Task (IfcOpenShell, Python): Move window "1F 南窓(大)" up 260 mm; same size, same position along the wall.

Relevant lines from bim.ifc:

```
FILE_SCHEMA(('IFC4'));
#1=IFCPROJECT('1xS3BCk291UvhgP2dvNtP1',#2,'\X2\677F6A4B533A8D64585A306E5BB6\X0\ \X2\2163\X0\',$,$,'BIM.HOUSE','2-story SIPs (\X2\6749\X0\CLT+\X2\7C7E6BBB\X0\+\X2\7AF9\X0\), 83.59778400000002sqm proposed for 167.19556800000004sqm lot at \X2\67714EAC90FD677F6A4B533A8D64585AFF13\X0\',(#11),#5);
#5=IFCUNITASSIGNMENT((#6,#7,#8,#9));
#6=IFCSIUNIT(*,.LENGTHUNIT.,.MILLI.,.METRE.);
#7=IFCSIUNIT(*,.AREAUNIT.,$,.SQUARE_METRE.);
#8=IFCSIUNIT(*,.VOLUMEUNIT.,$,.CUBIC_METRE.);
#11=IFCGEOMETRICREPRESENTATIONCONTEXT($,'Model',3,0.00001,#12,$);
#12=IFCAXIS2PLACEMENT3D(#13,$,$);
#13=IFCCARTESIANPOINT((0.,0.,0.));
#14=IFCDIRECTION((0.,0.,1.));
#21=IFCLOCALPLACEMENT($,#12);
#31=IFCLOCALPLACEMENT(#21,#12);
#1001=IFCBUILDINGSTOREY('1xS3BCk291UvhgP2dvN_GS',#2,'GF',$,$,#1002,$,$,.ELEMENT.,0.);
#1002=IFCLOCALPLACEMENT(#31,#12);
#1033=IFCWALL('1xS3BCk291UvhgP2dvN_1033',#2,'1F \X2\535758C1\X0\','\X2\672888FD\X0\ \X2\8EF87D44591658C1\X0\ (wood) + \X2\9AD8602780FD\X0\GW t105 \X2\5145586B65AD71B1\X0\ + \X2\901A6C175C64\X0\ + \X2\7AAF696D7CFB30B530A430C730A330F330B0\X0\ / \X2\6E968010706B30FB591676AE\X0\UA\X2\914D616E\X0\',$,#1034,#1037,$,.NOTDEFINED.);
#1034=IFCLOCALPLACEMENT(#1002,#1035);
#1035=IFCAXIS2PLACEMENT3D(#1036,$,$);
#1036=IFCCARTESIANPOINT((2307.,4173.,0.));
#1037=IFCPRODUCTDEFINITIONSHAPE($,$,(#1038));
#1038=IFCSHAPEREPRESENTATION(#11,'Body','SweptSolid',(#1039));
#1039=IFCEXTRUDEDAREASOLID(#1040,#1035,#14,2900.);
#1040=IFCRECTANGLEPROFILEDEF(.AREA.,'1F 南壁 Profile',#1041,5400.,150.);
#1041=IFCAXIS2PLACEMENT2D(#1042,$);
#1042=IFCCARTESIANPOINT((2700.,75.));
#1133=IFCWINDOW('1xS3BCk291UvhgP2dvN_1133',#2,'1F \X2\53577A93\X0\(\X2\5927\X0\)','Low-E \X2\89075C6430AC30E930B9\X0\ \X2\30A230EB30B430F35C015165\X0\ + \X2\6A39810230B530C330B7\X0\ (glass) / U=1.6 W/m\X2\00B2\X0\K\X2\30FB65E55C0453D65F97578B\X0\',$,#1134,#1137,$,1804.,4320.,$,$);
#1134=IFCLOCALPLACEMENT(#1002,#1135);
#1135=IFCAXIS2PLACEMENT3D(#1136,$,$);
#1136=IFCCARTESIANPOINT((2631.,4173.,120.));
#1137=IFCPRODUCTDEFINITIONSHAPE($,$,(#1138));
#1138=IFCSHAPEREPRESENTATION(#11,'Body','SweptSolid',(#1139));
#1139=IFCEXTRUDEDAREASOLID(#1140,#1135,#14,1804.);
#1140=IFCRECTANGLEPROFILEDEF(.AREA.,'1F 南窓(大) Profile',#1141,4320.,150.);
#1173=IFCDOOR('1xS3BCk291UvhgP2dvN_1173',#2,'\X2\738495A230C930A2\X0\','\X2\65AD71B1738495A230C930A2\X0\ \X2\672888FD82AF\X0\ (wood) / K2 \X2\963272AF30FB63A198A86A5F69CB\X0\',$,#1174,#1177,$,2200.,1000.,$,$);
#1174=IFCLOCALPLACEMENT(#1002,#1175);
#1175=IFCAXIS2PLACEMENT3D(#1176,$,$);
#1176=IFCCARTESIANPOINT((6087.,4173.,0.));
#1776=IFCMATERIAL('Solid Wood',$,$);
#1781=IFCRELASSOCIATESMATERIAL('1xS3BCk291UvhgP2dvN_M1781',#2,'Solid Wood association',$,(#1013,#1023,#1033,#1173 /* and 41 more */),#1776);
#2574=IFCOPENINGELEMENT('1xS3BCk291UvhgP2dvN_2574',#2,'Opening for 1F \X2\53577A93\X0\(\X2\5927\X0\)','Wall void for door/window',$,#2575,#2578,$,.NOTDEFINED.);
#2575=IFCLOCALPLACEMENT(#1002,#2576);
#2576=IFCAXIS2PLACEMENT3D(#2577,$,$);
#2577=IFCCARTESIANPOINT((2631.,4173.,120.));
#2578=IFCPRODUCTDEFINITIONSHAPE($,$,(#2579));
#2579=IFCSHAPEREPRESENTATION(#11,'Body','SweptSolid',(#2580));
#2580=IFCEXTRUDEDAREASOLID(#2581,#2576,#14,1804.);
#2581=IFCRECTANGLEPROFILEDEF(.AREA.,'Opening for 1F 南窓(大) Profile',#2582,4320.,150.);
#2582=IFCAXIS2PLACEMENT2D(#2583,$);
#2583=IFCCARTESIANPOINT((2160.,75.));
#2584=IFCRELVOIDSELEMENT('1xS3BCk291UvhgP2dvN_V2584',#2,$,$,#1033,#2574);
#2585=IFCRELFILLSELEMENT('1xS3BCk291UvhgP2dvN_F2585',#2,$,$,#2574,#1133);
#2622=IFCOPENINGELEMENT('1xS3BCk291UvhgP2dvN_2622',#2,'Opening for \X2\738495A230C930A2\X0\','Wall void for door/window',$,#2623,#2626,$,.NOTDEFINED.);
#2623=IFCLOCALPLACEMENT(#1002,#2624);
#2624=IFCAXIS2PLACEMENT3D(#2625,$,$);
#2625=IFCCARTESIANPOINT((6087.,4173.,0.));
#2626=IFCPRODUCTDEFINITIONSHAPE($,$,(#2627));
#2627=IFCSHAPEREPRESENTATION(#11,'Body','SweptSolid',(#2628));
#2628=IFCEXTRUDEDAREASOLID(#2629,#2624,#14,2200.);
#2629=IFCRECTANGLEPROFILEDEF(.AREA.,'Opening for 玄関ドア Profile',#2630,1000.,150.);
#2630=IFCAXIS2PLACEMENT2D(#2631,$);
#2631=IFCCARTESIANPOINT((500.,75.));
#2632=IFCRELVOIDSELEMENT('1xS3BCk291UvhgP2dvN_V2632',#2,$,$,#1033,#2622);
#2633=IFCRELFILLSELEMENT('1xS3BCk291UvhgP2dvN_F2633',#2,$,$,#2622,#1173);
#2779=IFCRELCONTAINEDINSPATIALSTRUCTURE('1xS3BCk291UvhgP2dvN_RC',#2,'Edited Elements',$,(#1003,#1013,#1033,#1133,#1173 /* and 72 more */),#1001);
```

```python
import numpy as np
import ifcopenshell
import ifcopenshell.api.geometry
import ifcopenshell.util.placement
import ifcopenshell.util.unit

model = ifcopenshell.open("bim.ifc")
unit_scale = ifcopenshell.util.unit.calculate_unit_scale(model)

window = model.by_guid("1xS3BCk291UvhgP2dvN_1133")
opening = window.FillsVoids[0].RelatingOpeningElement
dz = 0.26 / unit_scale

shift = np.array([0.0, 0.0, dz])
# The window is not placed relative to its opening, so move both.
for product in (opening, window):
    matrix = ifcopenshell.util.placement.get_local_placement(product.ObjectPlacement)
    matrix[:3, 3] += shift
    ifcopenshell.api.geometry.edit_object_placement(model, product=product, matrix=matrix, is_si=False)

print(f"moved by {dz * unit_scale:+.3f} m")

model.write("bim_updated.ifc")
```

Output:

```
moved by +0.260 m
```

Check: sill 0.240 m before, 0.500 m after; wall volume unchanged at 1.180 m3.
